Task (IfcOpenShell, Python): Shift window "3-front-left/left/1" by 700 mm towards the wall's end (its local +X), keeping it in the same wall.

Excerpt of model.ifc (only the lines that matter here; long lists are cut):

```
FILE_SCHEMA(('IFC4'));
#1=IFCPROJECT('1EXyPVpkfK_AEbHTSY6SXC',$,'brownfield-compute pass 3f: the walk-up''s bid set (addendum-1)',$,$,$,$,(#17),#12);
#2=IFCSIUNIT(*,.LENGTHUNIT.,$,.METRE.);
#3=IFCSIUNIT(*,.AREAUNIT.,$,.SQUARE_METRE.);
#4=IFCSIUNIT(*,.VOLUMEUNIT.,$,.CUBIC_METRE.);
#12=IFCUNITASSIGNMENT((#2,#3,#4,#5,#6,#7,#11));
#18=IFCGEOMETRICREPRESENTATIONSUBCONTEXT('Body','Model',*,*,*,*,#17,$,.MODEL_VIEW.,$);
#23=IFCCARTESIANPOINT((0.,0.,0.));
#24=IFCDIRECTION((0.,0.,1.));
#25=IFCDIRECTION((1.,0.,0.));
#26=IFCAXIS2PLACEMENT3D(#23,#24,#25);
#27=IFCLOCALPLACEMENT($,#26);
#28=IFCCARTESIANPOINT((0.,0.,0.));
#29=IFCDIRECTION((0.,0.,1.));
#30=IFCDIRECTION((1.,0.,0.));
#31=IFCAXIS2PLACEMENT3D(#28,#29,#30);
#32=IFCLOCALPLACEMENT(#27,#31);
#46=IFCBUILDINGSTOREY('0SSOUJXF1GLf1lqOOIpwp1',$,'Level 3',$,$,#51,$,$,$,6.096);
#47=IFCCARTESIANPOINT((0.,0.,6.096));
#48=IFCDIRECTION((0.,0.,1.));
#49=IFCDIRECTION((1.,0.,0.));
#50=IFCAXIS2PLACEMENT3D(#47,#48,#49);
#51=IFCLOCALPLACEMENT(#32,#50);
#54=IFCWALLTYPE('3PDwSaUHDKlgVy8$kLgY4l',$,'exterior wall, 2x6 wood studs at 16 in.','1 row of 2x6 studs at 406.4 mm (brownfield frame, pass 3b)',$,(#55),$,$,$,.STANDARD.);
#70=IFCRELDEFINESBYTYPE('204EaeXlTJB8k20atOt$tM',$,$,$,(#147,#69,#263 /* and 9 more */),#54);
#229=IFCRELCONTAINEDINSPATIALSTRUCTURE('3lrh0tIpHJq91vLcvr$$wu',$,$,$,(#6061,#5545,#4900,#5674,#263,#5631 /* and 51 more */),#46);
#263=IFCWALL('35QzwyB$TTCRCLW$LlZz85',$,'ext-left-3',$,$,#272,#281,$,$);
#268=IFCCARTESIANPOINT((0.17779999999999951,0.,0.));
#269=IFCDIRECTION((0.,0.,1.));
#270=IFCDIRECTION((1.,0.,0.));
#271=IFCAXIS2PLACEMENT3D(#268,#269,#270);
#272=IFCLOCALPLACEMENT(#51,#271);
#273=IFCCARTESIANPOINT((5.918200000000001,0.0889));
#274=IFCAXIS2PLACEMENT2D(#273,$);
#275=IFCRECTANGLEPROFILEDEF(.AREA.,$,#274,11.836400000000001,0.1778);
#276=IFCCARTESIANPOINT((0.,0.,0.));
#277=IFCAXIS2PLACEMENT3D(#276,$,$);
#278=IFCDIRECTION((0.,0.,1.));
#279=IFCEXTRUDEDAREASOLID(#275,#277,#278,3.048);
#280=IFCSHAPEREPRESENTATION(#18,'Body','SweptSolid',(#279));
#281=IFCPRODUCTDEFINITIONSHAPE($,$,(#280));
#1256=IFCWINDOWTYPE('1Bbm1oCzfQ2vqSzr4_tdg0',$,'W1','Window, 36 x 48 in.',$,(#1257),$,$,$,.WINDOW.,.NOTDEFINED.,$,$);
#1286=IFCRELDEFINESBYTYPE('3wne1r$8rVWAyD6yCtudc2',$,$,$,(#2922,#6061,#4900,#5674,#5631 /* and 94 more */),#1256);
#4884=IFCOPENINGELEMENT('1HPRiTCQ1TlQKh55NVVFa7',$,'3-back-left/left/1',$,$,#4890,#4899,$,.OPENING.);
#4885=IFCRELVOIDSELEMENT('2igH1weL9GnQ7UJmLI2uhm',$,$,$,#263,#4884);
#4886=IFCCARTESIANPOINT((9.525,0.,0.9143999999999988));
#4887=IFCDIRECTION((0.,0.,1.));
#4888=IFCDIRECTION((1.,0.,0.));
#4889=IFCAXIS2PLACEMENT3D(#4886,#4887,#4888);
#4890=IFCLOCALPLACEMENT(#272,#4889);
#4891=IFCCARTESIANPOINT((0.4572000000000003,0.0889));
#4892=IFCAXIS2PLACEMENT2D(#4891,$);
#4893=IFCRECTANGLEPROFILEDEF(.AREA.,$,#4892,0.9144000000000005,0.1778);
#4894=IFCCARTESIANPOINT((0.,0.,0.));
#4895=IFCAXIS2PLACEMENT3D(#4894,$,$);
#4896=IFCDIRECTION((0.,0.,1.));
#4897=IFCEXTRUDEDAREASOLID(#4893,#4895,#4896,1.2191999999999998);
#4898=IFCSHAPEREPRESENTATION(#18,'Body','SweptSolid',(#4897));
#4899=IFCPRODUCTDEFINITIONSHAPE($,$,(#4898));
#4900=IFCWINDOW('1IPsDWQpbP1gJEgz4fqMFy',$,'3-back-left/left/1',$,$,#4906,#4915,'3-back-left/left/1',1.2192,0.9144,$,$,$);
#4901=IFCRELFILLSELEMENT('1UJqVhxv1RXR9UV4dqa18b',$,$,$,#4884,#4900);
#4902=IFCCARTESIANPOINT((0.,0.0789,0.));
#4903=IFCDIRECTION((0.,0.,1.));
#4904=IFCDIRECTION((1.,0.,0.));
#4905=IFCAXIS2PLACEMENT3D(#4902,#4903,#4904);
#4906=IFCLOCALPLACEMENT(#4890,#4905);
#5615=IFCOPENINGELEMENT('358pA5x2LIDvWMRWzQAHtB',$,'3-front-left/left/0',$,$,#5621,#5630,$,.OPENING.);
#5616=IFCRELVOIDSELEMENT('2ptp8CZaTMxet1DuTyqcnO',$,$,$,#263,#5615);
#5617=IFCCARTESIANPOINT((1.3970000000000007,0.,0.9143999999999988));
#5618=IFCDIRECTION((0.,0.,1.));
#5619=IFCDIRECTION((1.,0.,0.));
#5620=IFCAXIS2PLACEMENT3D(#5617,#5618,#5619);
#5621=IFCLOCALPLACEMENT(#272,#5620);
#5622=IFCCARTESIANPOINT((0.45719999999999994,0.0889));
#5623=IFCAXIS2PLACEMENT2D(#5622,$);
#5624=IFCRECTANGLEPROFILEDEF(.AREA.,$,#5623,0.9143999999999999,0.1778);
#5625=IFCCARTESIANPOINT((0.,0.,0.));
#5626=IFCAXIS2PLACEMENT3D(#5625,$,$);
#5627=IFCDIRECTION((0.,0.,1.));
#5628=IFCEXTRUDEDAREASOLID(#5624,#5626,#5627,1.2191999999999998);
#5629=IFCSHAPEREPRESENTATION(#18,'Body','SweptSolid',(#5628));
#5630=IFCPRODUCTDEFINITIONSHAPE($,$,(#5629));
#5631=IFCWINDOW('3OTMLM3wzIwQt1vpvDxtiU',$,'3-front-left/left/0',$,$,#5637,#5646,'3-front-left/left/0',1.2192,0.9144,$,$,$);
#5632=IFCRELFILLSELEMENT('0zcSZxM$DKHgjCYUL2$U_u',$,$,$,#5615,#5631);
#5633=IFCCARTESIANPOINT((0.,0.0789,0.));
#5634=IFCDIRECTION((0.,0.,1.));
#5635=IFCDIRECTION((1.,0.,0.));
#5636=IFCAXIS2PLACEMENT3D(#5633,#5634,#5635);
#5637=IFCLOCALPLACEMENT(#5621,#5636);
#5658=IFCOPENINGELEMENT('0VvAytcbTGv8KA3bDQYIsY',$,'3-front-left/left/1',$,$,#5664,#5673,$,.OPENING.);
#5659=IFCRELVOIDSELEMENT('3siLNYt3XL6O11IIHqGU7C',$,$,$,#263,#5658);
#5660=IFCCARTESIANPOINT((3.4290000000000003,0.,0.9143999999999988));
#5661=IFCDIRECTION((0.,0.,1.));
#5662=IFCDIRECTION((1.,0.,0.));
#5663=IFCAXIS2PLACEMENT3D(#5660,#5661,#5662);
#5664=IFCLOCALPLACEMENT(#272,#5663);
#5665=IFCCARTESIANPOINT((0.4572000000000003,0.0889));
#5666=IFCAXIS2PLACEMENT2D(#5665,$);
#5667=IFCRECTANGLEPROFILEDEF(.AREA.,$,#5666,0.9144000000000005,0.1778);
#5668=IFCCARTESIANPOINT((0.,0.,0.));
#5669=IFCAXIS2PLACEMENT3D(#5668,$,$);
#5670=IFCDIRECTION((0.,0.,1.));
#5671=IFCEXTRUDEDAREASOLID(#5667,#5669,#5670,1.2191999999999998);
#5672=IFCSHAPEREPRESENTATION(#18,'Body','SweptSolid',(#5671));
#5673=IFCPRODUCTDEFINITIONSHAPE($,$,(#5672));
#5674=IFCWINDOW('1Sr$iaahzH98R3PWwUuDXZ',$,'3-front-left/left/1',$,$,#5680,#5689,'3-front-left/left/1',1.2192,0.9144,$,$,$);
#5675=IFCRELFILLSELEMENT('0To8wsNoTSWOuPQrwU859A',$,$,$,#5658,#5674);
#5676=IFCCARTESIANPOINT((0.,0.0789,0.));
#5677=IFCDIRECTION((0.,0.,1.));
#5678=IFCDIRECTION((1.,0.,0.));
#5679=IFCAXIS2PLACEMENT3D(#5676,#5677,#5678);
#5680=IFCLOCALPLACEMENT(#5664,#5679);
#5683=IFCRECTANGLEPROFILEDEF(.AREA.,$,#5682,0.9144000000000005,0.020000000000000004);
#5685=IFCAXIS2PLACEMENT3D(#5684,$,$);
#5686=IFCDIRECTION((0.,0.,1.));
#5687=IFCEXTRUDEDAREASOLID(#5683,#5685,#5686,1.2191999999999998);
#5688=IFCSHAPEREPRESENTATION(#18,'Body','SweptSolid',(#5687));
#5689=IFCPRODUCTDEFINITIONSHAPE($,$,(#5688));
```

```python
import ifcopenshell
import ifcopenshell.api.geometry
import ifcopenshell.util.placement
import ifcopenshell.util.unit

model = ifcopenshell.open("model.ifc")
unit_scale = ifcopenshell.util.unit.calculate_unit_scale(model)

window = model.by_guid("1Sr$iaahzH98R3PWwUuDXZ")
opening = window.FillsVoids[0].RelatingOpeningElement
wall = opening.VoidsElements[0].RelatingBuildingElement

wall_matrix = ifcopenshell.util.placement.get_local_placement(wall.ObjectPlacement)
shift = wall_matrix[:3, 0] * 0.7 / unit_scale
before = ifcopenshell.util.placement.get_local_placement(window.ObjectPlacement)[:3, 3].copy()

# The window is placed relative to its opening, so it follows when the opening moves.
matrix = ifcopenshell.util.placement.get_local_placement(opening.ObjectPlacement)
matrix[:3, 3] += shift
ifcopenshell.api.geometry.edit_object_placement(
    model, product=opening, matrix=matrix, is_si=False, should_transform_children=True
)

after = ifcopenshell.util.placement.get_local_placement(window.ObjectPlacement)[:3, 3]
print("window moved by", (after - before).round(3) + 0.0)

model.write("model_rev.ifc")
```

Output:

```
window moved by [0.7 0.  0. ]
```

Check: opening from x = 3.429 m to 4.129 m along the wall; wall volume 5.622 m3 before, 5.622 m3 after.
